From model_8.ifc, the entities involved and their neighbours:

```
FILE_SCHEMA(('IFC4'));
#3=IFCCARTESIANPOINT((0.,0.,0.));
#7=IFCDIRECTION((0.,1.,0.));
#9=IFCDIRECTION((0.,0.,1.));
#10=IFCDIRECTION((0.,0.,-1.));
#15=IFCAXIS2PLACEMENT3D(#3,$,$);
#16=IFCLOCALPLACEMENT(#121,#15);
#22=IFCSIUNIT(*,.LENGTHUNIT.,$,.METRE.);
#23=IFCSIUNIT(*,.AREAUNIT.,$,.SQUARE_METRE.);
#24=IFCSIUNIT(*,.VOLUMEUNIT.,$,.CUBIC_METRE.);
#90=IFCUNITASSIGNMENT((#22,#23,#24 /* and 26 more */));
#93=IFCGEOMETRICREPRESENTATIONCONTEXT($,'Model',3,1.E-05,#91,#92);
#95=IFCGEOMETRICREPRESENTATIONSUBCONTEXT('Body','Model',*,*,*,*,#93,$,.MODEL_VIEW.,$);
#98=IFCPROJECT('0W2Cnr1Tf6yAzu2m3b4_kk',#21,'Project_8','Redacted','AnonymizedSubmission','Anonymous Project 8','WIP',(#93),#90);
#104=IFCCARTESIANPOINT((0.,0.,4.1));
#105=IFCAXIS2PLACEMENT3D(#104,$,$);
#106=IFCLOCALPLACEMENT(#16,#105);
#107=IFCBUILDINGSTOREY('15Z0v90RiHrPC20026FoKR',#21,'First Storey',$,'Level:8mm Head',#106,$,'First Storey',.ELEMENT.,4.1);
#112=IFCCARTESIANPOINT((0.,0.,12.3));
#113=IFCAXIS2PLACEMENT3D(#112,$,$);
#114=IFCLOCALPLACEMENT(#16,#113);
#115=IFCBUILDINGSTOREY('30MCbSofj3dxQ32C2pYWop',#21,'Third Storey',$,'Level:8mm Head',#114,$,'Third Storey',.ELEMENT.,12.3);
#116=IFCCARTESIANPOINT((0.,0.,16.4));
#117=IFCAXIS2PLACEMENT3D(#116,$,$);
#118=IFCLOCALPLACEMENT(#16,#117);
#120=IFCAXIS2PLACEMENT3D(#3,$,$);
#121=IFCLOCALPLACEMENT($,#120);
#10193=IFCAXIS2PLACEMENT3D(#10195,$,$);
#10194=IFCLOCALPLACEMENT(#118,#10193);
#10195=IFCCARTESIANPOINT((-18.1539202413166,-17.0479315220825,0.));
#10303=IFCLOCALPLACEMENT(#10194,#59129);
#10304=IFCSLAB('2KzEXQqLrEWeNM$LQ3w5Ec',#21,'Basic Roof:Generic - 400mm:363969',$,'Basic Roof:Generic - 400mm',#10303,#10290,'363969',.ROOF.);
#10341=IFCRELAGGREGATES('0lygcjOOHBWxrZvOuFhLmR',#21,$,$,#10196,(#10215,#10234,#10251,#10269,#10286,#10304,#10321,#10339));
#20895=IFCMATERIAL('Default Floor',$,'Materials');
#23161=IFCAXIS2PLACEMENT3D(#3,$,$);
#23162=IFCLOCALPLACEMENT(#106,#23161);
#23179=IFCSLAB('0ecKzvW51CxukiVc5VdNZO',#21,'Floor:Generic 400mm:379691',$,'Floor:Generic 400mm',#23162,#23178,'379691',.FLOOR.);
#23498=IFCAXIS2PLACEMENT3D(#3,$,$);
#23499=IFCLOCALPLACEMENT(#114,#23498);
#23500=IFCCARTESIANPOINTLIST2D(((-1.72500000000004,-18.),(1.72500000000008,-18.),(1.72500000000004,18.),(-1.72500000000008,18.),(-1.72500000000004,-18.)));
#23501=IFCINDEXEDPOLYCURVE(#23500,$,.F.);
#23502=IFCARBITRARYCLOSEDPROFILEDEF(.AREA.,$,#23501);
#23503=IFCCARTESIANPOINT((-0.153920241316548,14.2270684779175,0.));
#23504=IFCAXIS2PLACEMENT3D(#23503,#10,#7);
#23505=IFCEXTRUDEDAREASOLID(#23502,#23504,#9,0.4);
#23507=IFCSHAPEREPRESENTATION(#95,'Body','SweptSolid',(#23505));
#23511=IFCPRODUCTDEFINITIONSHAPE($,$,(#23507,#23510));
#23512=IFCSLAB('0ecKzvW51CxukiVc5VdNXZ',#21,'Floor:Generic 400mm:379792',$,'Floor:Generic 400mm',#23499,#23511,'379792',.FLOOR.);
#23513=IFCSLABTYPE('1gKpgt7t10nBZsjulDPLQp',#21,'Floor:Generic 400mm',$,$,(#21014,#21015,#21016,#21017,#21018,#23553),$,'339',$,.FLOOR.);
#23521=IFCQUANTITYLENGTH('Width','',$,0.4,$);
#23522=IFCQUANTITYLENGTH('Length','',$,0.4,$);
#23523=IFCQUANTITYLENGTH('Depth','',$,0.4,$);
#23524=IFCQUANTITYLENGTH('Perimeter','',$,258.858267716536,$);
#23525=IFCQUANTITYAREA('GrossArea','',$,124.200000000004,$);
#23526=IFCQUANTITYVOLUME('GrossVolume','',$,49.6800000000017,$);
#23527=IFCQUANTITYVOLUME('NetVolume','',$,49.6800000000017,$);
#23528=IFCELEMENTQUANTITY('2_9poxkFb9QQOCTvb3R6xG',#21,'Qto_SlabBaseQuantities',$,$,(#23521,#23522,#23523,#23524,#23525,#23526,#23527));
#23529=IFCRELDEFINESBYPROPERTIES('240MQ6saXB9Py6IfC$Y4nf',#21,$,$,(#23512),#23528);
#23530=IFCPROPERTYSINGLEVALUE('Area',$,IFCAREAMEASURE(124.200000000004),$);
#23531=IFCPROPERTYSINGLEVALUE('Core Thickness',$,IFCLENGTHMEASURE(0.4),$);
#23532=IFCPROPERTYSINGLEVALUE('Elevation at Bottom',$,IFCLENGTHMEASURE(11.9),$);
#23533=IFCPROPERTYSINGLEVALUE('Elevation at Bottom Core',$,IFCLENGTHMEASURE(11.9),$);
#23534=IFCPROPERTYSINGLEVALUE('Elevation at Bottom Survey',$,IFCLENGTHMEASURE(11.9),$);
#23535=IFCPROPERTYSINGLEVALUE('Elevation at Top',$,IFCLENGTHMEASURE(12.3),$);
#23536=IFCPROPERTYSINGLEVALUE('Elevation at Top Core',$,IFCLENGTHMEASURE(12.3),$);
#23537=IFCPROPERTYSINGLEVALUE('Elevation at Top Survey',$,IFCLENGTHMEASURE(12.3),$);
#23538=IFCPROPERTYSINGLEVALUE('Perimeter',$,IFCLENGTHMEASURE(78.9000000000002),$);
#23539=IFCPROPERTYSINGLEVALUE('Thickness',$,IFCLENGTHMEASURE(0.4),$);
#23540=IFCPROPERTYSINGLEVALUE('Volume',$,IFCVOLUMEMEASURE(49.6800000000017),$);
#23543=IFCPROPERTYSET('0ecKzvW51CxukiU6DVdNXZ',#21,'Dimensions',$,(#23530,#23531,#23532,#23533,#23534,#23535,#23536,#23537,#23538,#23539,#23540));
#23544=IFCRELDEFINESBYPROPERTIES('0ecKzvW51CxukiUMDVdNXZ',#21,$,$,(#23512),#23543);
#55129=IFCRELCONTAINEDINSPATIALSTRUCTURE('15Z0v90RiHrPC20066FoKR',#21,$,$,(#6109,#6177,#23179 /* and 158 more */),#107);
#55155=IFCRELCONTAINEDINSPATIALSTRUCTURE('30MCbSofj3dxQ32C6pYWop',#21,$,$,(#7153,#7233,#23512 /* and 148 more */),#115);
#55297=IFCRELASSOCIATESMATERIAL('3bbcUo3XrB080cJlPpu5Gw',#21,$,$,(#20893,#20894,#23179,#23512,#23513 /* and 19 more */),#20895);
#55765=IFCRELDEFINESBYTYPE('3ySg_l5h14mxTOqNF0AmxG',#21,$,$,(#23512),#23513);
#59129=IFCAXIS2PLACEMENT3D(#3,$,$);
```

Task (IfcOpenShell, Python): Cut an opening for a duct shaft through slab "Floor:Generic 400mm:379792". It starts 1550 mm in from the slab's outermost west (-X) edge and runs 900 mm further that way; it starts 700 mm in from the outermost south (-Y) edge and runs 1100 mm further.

```python
import numpy as np
import ifcopenshell
import ifcopenshell.api.feature
import ifcopenshell.api.geometry
import ifcopenshell.api.pset
import ifcopenshell.api.root
import ifcopenshell.geom
import ifcopenshell.util.element
import ifcopenshell.util.placement
import ifcopenshell.util.representation
import ifcopenshell.util.shape
import ifcopenshell.util.unit

model = ifcopenshell.open("model_8.ifc")
unit_scale = ifcopenshell.util.unit.calculate_unit_scale(model)
area_scale = ifcopenshell.util.unit.calculate_unit_scale(model, "AREAUNIT")
volume_scale = ifcopenshell.util.unit.calculate_unit_scale(model, "VOLUMEUNIT")
settings = ifcopenshell.geom.settings()


def volume(element):
    """Net volume in cubic metres, openings subtracted."""
    shape = ifcopenshell.geom.create_shape(settings, element)
    return ifcopenshell.util.shape.get_volume(shape.geometry)


slab = model.by_guid("0ecKzvW51CxukiVc5VdNXZ")
before = volume(slab)

# Extent in the slab's own axes, in metres. The edges named are its -X and -Y sides.
slab_shape = ifcopenshell.geom.create_shape(settings, slab)
vertices = ifcopenshell.util.shape.get_vertices(slab_shape.geometry)
x_min, y_min, bottom = vertices.min(axis=0)
top = vertices[:, 2].max()

opening = ifcopenshell.api.root.create_entity(model, ifc_class="IfcOpeningElement", name="Duct shaft opening", predefined_type="OPENING")
context = ifcopenshell.util.representation.get_context(model, "Model", "Body", "MODEL_VIEW")
width, depth = 0.9, 1.1
outline = [(0.0, 0.0), (width, 0.0), (width, depth), (0.0, depth), (0.0, 0.0)]
# Overshoot both faces by 50 mm so the cut is clean.
shape = ifcopenshell.api.geometry.add_slab_representation(
    model, context=context, depth=top - bottom + 0.1, polyline=outline
)
ifcopenshell.api.geometry.assign_representation(model, product=opening, representation=shape)

matrix = ifcopenshell.util.placement.get_local_placement(slab.ObjectPlacement)
matrix[:, 3] = matrix @ np.append(np.array([x_min + 1.55, y_min + 0.7, bottom - 0.05]) / unit_scale, 1.0)
ifcopenshell.api.geometry.edit_object_placement(model, product=opening, matrix=matrix, is_si=False)
ifcopenshell.api.feature.add_feature(model, feature=opening, element=slab)

after = volume(slab)

# Update the slab's stored quantities.
qto = model.by_id(ifcopenshell.util.element.get_pset(slab, "Qto_SlabBaseQuantities", should_inherit=False)["id"])
ifcopenshell.api.pset.edit_qto(model, qto=qto, properties={"NetVolume": after / volume_scale})
pset = model.by_id(ifcopenshell.util.element.get_pset(slab, "Dimensions", should_inherit=False)["id"])
ifcopenshell.api.pset.edit_pset(model, pset=pset, properties={
    "Area": model.create_entity("IfcAreaMeasure", after / (top - bottom) / area_scale),
    "Volume": model.create_entity("IfcVolumeMeasure", after / volume_scale),
})

print(f"slab volume {before:.3f} -> {after:.3f} m3")

model.write("model_8_updated.ifc")
```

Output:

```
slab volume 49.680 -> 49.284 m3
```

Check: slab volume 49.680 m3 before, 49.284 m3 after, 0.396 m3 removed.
